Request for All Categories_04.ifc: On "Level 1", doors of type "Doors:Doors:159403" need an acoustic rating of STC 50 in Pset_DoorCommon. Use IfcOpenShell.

First a look at what the model holds.

```python
import ifcopenshell
import ifcopenshell.util.element

model = ifcopenshell.open("All Categories_04.ifc")
print(model.schema)
storey = next(s for s in model.by_type("IfcBuildingStorey") if s.Name == "Level 1")
doors = [e for e in ifcopenshell.util.element.get_decomposition(storey) if e.is_a("IfcDoor")]
seen = {}
for e in doors:
    element_type = ifcopenshell.util.element.get_type(e)
    key = (element_type.Name if element_type != e and element_type else None, ifcopenshell.util.element.get_pset(e, "Pset_DoorCommon", "AcousticRating"))
    seen[key] = seen.get(key, 0) + 1
for (name, value), count in sorted(seen.items(), key=str):
    print(count, "x", name, "|", value)
```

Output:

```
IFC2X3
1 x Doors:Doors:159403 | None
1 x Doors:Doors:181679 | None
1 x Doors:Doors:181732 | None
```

```python
import ifcopenshell
import ifcopenshell.api.pset
import ifcopenshell.util.element

model = ifcopenshell.open("All Categories_04.ifc")

storey = next(s for s in model.by_type("IfcBuildingStorey") if s.Name == "Level 1")
doors = [e for e in ifcopenshell.util.element.get_decomposition(storey) if e.is_a("IfcDoor")]

count = 0
for e in doors:
    element_type = ifcopenshell.util.element.get_type(e)
    if element_type in (None, e) or element_type.Name != "Doors:Doors:159403":
        continue
    # add_pset returns the element's existing set when there is one.
    pset = ifcopenshell.api.pset.add_pset(model, product=e, name="Pset_DoorCommon")
    ifcopenshell.api.pset.edit_pset(model, pset=pset, properties={"AcousticRating": "STC 50"})
    count += 1

print(count, "doors updated")

model.write("All Categories_04_rev.ifc")
```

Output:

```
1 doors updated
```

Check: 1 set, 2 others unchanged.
